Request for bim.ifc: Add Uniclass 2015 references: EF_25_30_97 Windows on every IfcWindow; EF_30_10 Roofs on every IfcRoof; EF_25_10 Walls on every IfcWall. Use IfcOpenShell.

First a look at what the model holds.

```python
import ifcopenshell

model = ifcopenshell.open("bim.ifc")
print(model.schema)
print("classifications:", [c.Name for c in model.by_type("IfcClassification")])
for ifc_class in ("IfcDoor", "IfcRoof", "IfcStair", "IfcWall", "IfcWindow"):
    print(ifc_class, len(model.by_type(ifc_class)))
```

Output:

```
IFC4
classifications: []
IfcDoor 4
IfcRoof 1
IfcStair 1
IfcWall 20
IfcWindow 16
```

```python
import ifcopenshell
import ifcopenshell.api.classification

model = ifcopenshell.open("bim.ifc")

system = ifcopenshell.api.classification.add_classification(model, classification="Uniclass 2015")

codes = {
    "IfcWindow": ("EF_25_30_97", "Windows"),
    "IfcRoof": ("EF_30_10", "Roofs"),
    "IfcWall": ("EF_25_10", "Walls"),
}
for ifc_class, (code, name) in codes.items():
    products = model.by_type(ifc_class)
    ifcopenshell.api.classification.add_reference(
        model, products=products, classification=system, identification=code, name=name
    )
    print(code, len(products))

model.write("bim_rev.ifc")
```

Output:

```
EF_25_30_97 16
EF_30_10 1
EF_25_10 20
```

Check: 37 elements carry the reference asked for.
